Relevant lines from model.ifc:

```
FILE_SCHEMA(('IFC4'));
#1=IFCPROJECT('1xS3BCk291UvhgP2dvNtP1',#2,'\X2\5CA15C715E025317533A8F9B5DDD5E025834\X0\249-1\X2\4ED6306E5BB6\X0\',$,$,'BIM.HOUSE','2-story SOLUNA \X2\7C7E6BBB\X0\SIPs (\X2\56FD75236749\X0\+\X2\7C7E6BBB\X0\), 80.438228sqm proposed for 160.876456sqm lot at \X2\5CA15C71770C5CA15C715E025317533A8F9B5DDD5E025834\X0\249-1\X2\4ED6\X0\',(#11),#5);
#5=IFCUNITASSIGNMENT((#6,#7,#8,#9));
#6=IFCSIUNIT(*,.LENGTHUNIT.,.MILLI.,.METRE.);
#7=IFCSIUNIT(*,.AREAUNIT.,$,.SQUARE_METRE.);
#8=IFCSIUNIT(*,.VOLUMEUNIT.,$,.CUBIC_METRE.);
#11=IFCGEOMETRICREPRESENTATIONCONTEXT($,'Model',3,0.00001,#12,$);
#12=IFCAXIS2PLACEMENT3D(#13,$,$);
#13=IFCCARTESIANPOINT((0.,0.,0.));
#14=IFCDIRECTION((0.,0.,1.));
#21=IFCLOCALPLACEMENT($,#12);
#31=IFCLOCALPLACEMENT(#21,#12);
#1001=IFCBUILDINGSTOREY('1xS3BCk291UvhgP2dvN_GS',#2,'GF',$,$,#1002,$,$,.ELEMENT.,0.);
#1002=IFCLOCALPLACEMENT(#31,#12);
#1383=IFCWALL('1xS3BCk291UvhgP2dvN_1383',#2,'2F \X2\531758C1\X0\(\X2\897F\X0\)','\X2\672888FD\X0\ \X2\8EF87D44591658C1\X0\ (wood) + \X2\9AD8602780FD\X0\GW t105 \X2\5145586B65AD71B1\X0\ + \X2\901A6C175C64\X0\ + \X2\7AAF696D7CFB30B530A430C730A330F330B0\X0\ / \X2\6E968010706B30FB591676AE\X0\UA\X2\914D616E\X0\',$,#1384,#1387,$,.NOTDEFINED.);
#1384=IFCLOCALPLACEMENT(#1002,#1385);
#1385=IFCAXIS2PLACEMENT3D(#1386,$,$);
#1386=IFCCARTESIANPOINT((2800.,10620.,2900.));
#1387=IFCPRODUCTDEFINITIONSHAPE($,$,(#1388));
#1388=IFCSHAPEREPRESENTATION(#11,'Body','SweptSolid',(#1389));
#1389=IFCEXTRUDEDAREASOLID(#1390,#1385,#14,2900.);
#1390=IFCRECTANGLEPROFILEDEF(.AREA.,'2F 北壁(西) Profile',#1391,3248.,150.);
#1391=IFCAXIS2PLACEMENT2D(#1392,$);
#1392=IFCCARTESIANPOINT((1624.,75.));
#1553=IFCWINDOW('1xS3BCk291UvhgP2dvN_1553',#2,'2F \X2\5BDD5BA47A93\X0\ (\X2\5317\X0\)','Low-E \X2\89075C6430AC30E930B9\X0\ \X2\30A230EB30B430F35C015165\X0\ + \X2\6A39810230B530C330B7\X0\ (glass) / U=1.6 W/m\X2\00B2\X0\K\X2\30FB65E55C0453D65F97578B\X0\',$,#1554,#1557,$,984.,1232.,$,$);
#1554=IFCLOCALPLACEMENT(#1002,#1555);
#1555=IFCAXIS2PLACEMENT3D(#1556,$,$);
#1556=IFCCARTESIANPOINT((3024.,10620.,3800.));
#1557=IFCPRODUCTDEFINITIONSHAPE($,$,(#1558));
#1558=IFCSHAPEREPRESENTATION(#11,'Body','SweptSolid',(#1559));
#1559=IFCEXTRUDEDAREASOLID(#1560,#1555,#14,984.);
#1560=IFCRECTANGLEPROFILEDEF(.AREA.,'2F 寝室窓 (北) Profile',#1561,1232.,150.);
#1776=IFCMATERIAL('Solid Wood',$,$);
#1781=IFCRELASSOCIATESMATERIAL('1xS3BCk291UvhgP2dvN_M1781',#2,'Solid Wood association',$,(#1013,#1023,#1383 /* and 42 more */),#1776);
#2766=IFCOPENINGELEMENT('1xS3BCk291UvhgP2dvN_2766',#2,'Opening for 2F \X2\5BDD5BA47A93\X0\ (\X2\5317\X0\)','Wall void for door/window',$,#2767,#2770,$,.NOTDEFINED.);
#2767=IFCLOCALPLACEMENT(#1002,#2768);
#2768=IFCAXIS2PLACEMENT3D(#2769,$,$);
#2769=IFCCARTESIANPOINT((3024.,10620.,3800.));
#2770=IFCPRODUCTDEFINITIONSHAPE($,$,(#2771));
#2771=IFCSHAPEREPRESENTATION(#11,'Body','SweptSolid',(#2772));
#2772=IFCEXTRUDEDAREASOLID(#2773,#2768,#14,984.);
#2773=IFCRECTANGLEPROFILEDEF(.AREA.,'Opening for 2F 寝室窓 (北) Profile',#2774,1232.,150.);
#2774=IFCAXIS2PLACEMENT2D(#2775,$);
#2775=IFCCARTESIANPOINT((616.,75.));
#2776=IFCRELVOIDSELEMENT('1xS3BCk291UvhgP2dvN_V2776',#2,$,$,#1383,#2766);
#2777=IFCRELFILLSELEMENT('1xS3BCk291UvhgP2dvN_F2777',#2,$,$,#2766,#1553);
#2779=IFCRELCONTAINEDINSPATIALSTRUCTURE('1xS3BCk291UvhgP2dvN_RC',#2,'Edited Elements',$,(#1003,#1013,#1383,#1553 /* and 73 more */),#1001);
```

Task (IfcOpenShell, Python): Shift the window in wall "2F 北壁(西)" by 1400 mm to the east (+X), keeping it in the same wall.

```python
import ifcopenshell
import ifcopenshell.api.geometry
import ifcopenshell.util.placement

model = ifcopenshell.open("model.ifc")

window = model.by_guid("1xS3BCk291UvhgP2dvN_1553")
opening = window.FillsVoids[0].RelatingOpeningElement
wall = opening.VoidsElements[0].RelatingBuildingElement

wall_matrix = ifcopenshell.util.placement.get_local_placement(wall.ObjectPlacement)
shift = wall_matrix[:3, 0] * 1400.0
before = ifcopenshell.util.placement.get_local_placement(window.ObjectPlacement)[:3, 3].copy()

# The window is not placed relative to its opening, so move both.
for product in (opening, window):
    matrix = ifcopenshell.util.placement.get_local_placement(product.ObjectPlacement)
    matrix[:3, 3] += shift
    ifcopenshell.api.geometry.edit_object_placement(model, product=product, matrix=matrix, is_si=False)

after = ifcopenshell.util.placement.get_local_placement(window.ObjectPlacement)[:3, 3]
print("window moved by", (after - before).round(3) + 0.0)

model.write("model_v2.ifc")
```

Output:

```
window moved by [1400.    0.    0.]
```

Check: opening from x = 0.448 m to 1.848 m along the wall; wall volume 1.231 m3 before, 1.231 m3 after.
